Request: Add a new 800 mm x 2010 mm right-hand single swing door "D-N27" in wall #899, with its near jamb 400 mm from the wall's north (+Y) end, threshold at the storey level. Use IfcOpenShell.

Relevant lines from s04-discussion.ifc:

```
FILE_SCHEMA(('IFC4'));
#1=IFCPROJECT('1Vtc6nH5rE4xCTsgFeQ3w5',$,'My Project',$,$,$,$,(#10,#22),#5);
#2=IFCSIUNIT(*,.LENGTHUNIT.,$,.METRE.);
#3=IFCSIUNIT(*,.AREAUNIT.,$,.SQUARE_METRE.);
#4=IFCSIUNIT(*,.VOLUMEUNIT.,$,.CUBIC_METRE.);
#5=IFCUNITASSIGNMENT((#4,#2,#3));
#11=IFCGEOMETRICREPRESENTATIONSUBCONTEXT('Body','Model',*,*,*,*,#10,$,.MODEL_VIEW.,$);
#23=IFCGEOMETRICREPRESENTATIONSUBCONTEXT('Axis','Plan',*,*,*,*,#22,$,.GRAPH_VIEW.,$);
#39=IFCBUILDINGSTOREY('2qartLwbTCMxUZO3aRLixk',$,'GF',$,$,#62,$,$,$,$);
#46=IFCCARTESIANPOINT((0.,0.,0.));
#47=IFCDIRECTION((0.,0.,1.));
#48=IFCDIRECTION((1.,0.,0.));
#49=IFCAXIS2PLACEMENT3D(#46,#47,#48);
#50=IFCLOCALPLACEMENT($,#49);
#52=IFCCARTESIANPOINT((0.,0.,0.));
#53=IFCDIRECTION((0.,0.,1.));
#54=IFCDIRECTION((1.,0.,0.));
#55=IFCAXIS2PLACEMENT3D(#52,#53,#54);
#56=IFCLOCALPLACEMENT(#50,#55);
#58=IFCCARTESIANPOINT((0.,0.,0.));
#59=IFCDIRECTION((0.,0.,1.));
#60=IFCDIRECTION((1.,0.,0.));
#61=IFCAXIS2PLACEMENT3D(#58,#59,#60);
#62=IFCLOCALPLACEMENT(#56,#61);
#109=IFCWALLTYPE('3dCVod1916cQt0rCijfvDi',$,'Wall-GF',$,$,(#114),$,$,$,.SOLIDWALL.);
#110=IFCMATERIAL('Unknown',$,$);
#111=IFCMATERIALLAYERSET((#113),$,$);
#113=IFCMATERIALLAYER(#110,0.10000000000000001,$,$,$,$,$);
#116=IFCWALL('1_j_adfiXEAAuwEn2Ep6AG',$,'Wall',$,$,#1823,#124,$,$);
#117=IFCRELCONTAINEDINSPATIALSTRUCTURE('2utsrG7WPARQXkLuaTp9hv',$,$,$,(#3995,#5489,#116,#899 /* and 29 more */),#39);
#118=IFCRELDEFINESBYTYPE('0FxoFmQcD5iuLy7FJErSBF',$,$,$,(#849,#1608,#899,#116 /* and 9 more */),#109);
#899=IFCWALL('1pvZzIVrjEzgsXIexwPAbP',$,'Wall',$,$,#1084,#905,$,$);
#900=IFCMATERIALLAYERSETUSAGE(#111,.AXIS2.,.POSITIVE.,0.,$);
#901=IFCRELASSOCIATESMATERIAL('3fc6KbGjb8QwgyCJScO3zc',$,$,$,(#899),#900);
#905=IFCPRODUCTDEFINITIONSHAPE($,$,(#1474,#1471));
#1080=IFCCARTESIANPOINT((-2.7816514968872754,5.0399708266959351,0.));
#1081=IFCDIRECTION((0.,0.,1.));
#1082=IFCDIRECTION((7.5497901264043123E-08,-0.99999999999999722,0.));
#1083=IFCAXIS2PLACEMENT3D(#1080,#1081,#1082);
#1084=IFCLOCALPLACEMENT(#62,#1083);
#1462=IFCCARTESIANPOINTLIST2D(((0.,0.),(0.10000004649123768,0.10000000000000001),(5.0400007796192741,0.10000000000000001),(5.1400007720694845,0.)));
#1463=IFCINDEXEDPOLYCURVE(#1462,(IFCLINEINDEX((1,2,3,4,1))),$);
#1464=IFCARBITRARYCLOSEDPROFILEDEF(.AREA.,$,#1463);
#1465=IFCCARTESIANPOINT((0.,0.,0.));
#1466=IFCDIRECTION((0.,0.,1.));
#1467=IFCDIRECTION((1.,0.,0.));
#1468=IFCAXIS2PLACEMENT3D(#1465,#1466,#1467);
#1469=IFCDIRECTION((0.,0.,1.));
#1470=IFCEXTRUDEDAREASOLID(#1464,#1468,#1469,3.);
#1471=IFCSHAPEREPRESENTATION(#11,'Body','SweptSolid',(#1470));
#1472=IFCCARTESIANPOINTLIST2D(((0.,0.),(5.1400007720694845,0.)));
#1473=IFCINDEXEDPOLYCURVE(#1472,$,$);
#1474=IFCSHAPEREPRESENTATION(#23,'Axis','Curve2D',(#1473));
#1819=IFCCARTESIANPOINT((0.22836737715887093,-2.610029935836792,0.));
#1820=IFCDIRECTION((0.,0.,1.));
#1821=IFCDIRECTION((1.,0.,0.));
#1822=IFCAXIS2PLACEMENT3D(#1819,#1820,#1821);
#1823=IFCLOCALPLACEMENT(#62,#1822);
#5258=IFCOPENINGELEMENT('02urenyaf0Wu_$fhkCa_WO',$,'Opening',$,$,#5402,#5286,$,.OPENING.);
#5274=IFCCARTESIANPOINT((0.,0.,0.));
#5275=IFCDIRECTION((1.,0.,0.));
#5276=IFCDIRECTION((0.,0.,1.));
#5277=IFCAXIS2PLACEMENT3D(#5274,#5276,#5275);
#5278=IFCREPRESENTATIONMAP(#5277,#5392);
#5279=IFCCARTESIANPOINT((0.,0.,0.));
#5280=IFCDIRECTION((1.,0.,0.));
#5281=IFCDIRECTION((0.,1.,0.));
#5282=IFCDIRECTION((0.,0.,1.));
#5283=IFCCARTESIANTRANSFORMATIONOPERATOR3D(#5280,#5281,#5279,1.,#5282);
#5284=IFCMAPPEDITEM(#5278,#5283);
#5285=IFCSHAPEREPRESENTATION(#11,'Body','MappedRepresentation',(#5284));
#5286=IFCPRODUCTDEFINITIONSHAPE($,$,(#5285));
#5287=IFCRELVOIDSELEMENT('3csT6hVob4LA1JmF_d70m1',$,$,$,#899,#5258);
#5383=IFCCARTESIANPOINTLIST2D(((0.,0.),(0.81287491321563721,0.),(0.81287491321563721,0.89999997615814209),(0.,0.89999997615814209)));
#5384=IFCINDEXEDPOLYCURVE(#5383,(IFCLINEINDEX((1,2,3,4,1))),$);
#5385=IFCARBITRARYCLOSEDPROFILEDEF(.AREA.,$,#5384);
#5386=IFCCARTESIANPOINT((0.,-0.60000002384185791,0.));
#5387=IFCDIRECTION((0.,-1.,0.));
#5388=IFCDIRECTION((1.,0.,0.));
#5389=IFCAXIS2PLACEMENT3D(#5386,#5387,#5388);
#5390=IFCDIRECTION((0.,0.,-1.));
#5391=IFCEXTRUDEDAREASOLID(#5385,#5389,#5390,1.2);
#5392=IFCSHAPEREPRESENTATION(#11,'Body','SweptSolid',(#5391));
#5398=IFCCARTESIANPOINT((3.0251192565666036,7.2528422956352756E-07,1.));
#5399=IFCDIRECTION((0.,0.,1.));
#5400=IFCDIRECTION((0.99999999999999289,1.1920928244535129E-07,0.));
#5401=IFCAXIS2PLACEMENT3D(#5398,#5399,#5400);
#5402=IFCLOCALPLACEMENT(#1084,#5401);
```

```python
import numpy as np
import ifcopenshell
import ifcopenshell.api.feature
import ifcopenshell.api.geometry
import ifcopenshell.api.root
import ifcopenshell.api.spatial
import ifcopenshell.geom
import ifcopenshell.util.element
import ifcopenshell.util.placement
import ifcopenshell.util.representation
import ifcopenshell.util.shape
import ifcopenshell.util.unit

model = ifcopenshell.open("s04-discussion.ifc")
unit_scale = ifcopenshell.util.unit.calculate_unit_scale(model)
settings = ifcopenshell.geom.settings()


def volume(element):
    """Net volume in cubic metres, openings subtracted."""
    shape = ifcopenshell.geom.create_shape(settings, element)
    return ifcopenshell.util.shape.get_volume(shape.geometry)


wall = model.by_id(899)
storey = ifcopenshell.util.element.get_container(wall, ifc_class="IfcBuildingStorey")
context = ifcopenshell.util.representation.get_context(model, "Model", "Body", "MODEL_VIEW")
before = volume(wall)

width, height, from_end, sill = 0.8, 2.01, 0.4, 0.0  # metres

# The wall runs along its own X axis, and the end named is its -X end.
wall_shape = ifcopenshell.geom.create_shape(settings, wall)
x, y, z = ifcopenshell.util.shape.get_vertices(wall_shape.geometry).T
start = x.min() + from_end
face, thickness = float(y.min()), float(y.max() - y.min())
wall_matrix = ifcopenshell.util.placement.get_local_placement(wall.ObjectPlacement)
level = ifcopenshell.util.placement.get_local_placement(storey.ObjectPlacement)[2, 3]


def in_wall(x, y):
    """Placement at x, y metres in the wall's axes, at sill height."""
    matrix = wall_matrix.copy()
    matrix[:, 3] = wall_matrix @ np.array([x / unit_scale, y / unit_scale, 0.0, 1.0])
    matrix[2, 3] = level + sill / unit_scale
    return matrix


# Opening: a box that overshoots both wall faces by 50 mm.
opening = ifcopenshell.api.root.create_entity(model, ifc_class="IfcOpeningElement", predefined_type="OPENING")
box = ifcopenshell.api.geometry.add_wall_representation(
    model, context=context, length=width, height=height, thickness=thickness + 0.1
)
ifcopenshell.api.geometry.assign_representation(model, product=opening, representation=box)
ifcopenshell.api.geometry.edit_object_placement(model, product=opening, matrix=in_wall(start, face - 0.05), is_si=False)
ifcopenshell.api.feature.add_feature(model, feature=opening, element=wall)

door = ifcopenshell.api.root.create_entity(model, ifc_class="IfcDoor", name="D-N27", predefined_type="DOOR")
door.OverallWidth, door.OverallHeight = width / unit_scale, height / unit_scale
door.OperationType = "SINGLE_SWING_RIGHT"
body = ifcopenshell.api.geometry.add_door_representation(
    model,
    context=context,
    overall_width=door.OverallWidth,
    overall_height=door.OverallHeight,
    operation_type="SINGLE_SWING_RIGHT",
    lining_properties={"LiningDepth": thickness / unit_scale, "ThresholdDepth": thickness / unit_scale},
)
ifcopenshell.api.geometry.assign_representation(model, product=door, representation=body)
ifcopenshell.api.spatial.assign_container(model, products=[door], relating_structure=storey)
ifcopenshell.api.feature.add_filling(model, opening=opening, element=door)

# The lining spans the wall, so the door starts at the wall face.
ifcopenshell.api.geometry.edit_object_placement(model, product=door, matrix=in_wall(start, face), is_si=False)

after = volume(wall)

print(f"wall volume {before:.3f} -> {after:.3f} m3")

model.write("s04-discussion_rev.ifc")
```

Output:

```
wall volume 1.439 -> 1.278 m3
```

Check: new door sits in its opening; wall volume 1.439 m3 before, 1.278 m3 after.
